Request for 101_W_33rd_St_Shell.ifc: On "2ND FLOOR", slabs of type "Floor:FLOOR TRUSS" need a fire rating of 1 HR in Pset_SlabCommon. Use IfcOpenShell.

First a look at what the model holds.

```python
import ifcopenshell
import ifcopenshell.util.element

model = ifcopenshell.open("101_W_33rd_St_Shell.ifc")
print(model.schema)
storey = next(s for s in model.by_type("IfcBuildingStorey") if s.Name == "2ND FLOOR")
slabs = [e for e in ifcopenshell.util.element.get_decomposition(storey) if e.is_a("IfcSlab")]
seen = {}
for e in slabs:
    element_type = ifcopenshell.util.element.get_type(e)
    key = (element_type.Name if element_type != e and element_type else None, ifcopenshell.util.element.get_pset(e, "Pset_SlabCommon", "FireRating"))
    seen[key] = seen.get(key, 0) + 1
for (name, value), count in sorted(seen.items(), key=str):
    print(count, "x", name, "|", value)
```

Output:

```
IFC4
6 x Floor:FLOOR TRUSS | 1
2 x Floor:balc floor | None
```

```python
import ifcopenshell
import ifcopenshell.api.pset
import ifcopenshell.util.element

model = ifcopenshell.open("101_W_33rd_St_Shell.ifc")

storey = next(s for s in model.by_type("IfcBuildingStorey") if s.Name == "2ND FLOOR")
slabs = [e for e in ifcopenshell.util.element.get_decomposition(storey) if e.is_a("IfcSlab")]

count = 0
for e in slabs:
    element_type = ifcopenshell.util.element.get_type(e)
    if element_type in (None, e) or element_type.Name != "Floor:FLOOR TRUSS":
        continue
    # add_pset returns the element's existing set when there is one.
    pset = ifcopenshell.api.pset.add_pset(model, product=e, name="Pset_SlabCommon")
    ifcopenshell.api.pset.edit_pset(model, pset=pset, properties={"FireRating": "1 HR"})
    count += 1

print(count, "slabs updated")

model.write("101_W_33rd_St_Shell_v2.ifc")
```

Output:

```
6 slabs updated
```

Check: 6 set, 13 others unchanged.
